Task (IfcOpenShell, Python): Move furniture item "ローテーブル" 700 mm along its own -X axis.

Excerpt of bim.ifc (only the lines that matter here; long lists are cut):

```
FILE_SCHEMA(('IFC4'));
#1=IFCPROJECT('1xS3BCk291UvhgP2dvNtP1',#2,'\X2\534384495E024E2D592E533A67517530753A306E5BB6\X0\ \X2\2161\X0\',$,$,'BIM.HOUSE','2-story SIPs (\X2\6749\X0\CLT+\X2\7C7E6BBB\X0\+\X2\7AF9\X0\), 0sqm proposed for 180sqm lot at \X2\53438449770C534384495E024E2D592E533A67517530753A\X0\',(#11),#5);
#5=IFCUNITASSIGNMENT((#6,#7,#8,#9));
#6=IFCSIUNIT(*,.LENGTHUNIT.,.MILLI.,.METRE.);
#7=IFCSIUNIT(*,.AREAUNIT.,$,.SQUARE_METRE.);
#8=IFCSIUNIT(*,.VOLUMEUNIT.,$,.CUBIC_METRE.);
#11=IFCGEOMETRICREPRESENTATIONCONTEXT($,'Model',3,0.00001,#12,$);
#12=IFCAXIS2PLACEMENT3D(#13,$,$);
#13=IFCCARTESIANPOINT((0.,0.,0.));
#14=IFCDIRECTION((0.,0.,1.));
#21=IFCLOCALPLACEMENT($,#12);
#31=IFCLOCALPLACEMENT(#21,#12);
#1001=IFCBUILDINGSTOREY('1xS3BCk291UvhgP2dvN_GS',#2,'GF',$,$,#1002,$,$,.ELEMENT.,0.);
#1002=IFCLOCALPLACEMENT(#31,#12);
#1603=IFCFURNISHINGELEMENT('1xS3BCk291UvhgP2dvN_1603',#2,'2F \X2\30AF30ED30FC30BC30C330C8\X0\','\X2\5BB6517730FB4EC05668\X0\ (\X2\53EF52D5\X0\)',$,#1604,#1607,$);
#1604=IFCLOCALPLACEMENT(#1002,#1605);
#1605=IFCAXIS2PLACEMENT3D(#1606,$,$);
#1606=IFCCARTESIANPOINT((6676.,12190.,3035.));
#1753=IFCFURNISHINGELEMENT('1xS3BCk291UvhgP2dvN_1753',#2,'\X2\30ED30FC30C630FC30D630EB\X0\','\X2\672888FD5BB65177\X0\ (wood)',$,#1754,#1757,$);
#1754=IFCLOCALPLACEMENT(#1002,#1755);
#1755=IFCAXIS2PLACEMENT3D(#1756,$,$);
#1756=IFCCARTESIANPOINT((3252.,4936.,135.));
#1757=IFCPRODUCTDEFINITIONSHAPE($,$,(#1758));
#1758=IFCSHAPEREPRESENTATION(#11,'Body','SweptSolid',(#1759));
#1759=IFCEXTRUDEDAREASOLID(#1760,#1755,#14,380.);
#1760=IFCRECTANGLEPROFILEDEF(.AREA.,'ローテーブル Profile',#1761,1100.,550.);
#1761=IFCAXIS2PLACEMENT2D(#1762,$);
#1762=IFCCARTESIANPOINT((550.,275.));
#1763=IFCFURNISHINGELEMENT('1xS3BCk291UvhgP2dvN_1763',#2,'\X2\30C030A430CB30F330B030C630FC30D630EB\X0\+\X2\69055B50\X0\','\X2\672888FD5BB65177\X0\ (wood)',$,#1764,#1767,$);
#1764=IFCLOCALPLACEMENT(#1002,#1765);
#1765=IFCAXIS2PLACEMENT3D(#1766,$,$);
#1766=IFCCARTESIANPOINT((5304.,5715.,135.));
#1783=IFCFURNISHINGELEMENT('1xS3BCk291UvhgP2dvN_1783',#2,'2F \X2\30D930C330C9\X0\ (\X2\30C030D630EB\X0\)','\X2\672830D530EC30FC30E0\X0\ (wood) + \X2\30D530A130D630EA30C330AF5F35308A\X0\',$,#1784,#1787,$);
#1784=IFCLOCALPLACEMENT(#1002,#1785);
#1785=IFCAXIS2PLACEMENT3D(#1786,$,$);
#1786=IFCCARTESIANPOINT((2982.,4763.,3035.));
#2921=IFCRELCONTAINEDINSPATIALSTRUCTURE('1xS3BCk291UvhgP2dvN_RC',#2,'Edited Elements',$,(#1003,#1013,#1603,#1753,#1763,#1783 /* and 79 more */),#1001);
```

```python
import ifcopenshell
import ifcopenshell.api.geometry
import ifcopenshell.util.placement

model = ifcopenshell.open("bim.ifc")

item = model.by_guid("1xS3BCk291UvhgP2dvN_1753")
matrix = ifcopenshell.util.placement.get_local_placement(item.ObjectPlacement)
matrix[:3, 3] -= matrix[:3, 0] * 700.0
ifcopenshell.api.geometry.edit_object_placement(model, product=item, matrix=matrix, is_si=False)

print(ifcopenshell.util.placement.get_local_placement(item.ObjectPlacement).round(3) + 0.0)

model.write("bim_v2.ifc")
```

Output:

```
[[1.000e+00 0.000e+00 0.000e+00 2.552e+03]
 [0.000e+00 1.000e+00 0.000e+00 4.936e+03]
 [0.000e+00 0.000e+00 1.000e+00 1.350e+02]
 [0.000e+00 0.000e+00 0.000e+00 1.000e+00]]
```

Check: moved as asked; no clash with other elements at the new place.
